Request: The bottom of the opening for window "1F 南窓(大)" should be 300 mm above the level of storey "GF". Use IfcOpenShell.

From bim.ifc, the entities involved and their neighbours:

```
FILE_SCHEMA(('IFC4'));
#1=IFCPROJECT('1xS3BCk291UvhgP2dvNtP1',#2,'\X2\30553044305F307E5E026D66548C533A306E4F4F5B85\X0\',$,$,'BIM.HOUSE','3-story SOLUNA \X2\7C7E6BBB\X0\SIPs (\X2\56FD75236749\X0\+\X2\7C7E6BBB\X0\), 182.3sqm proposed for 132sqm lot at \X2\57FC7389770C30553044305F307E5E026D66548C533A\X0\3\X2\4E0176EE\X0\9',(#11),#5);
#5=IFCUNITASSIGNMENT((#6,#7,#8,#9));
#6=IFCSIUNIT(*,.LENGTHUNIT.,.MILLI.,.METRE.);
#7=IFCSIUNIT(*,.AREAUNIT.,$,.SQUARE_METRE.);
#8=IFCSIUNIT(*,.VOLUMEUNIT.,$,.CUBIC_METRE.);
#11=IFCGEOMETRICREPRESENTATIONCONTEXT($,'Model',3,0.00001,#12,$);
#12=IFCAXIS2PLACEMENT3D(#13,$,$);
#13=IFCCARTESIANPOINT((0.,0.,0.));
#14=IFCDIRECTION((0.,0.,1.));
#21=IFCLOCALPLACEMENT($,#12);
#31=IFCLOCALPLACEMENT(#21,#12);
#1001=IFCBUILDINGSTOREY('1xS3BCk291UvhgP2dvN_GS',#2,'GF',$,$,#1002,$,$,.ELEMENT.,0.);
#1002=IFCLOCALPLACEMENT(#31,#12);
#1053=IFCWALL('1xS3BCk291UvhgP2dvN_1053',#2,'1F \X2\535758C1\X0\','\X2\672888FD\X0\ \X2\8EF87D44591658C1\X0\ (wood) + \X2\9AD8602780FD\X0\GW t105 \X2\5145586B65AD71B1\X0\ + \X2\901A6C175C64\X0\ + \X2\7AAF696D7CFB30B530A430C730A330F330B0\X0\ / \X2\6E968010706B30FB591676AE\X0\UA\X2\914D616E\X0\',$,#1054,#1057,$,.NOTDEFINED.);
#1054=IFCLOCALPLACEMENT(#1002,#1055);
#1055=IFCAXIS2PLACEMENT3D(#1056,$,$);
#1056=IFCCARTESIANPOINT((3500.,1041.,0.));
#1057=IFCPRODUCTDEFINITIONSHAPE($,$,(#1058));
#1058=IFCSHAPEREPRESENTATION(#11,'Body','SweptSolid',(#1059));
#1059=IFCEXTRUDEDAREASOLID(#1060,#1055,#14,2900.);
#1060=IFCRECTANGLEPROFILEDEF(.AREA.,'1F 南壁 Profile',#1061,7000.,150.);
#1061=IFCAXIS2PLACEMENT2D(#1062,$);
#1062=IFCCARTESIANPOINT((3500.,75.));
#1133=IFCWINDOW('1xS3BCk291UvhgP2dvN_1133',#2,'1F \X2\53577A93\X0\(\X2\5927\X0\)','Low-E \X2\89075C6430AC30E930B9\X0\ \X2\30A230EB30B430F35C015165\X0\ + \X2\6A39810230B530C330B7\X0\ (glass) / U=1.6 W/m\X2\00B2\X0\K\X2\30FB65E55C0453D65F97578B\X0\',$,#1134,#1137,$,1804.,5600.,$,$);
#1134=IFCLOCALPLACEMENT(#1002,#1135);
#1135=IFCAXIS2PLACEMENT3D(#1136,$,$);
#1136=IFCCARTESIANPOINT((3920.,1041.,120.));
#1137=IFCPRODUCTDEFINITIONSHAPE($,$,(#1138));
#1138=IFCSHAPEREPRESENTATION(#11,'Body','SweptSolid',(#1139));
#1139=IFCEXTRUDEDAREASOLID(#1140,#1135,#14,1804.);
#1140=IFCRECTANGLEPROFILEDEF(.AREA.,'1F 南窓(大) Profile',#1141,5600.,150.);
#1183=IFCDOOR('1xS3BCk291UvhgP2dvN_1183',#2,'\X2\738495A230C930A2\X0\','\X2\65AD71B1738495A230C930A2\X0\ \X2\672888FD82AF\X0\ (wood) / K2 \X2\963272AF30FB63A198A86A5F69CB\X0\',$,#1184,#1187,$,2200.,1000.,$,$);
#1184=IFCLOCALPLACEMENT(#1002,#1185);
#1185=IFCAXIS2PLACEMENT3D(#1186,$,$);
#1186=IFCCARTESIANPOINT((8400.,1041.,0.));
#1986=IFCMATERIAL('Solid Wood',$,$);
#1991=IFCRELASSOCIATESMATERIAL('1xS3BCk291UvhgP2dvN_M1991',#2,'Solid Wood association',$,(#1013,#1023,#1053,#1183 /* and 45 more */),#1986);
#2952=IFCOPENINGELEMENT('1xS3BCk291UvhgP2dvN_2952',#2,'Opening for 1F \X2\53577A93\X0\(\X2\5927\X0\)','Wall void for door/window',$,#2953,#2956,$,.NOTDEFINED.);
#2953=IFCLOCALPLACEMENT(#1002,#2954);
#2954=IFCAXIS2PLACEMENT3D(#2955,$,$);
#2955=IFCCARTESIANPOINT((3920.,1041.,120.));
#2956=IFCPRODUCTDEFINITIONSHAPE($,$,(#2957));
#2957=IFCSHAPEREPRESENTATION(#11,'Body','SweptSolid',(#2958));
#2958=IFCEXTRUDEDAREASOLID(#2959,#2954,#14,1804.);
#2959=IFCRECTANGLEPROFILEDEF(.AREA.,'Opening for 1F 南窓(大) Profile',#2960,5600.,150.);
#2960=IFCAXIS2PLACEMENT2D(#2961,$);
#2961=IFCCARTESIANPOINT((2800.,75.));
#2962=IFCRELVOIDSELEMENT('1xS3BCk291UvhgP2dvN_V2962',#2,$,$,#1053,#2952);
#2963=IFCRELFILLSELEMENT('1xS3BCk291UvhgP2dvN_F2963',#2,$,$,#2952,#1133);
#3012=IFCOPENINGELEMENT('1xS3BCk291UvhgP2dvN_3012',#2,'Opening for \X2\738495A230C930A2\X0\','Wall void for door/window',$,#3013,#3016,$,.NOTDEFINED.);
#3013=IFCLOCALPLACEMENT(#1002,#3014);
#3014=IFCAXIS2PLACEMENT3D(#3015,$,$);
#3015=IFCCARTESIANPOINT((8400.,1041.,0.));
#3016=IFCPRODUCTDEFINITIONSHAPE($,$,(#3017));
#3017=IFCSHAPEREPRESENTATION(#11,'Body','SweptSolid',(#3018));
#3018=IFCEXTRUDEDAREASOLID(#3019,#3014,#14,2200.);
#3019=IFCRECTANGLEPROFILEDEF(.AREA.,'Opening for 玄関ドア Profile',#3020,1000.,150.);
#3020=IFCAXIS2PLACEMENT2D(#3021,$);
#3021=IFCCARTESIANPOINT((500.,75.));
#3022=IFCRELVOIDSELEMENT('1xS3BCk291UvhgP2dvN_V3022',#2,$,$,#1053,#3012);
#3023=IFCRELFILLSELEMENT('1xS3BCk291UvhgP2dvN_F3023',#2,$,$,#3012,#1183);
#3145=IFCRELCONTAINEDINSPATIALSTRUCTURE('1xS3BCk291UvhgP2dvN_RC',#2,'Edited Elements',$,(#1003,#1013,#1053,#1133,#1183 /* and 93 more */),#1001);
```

```python
import numpy as np
import ifcopenshell
import ifcopenshell.api.geometry
import ifcopenshell.geom
import ifcopenshell.util.element
import ifcopenshell.util.placement
import ifcopenshell.util.shape
import ifcopenshell.util.unit

model = ifcopenshell.open("bim.ifc")
unit_scale = ifcopenshell.util.unit.calculate_unit_scale(model)

window = model.by_id(1133)
opening = window.FillsVoids[0].RelatingOpeningElement
storey = ifcopenshell.util.element.get_container(window, ifc_class="IfcBuildingStorey")
level = ifcopenshell.util.placement.get_local_placement(storey.ObjectPlacement)[2, 3]

# The opening's origin need not be at the sill, so measure its lowest point.
shape = ifcopenshell.geom.create_shape(ifcopenshell.geom.settings(), opening)
bottom = ifcopenshell.util.shape.get_shape_bottom_elevation(shape, shape.geometry) / unit_scale
dz = level + 0.3 / unit_scale - bottom

shift = np.array([0.0, 0.0, dz])
# The window is not placed relative to its opening, so move both.
for product in (opening, window):
    matrix = ifcopenshell.util.placement.get_local_placement(product.ObjectPlacement)
    matrix[:3, 3] += shift
    ifcopenshell.api.geometry.edit_object_placement(model, product=product, matrix=matrix, is_si=False)

print(f"moved by {dz * unit_scale:+.3f} m")

model.write("bim_rev.ifc")
```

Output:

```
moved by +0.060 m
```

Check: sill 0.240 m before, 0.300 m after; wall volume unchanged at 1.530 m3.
